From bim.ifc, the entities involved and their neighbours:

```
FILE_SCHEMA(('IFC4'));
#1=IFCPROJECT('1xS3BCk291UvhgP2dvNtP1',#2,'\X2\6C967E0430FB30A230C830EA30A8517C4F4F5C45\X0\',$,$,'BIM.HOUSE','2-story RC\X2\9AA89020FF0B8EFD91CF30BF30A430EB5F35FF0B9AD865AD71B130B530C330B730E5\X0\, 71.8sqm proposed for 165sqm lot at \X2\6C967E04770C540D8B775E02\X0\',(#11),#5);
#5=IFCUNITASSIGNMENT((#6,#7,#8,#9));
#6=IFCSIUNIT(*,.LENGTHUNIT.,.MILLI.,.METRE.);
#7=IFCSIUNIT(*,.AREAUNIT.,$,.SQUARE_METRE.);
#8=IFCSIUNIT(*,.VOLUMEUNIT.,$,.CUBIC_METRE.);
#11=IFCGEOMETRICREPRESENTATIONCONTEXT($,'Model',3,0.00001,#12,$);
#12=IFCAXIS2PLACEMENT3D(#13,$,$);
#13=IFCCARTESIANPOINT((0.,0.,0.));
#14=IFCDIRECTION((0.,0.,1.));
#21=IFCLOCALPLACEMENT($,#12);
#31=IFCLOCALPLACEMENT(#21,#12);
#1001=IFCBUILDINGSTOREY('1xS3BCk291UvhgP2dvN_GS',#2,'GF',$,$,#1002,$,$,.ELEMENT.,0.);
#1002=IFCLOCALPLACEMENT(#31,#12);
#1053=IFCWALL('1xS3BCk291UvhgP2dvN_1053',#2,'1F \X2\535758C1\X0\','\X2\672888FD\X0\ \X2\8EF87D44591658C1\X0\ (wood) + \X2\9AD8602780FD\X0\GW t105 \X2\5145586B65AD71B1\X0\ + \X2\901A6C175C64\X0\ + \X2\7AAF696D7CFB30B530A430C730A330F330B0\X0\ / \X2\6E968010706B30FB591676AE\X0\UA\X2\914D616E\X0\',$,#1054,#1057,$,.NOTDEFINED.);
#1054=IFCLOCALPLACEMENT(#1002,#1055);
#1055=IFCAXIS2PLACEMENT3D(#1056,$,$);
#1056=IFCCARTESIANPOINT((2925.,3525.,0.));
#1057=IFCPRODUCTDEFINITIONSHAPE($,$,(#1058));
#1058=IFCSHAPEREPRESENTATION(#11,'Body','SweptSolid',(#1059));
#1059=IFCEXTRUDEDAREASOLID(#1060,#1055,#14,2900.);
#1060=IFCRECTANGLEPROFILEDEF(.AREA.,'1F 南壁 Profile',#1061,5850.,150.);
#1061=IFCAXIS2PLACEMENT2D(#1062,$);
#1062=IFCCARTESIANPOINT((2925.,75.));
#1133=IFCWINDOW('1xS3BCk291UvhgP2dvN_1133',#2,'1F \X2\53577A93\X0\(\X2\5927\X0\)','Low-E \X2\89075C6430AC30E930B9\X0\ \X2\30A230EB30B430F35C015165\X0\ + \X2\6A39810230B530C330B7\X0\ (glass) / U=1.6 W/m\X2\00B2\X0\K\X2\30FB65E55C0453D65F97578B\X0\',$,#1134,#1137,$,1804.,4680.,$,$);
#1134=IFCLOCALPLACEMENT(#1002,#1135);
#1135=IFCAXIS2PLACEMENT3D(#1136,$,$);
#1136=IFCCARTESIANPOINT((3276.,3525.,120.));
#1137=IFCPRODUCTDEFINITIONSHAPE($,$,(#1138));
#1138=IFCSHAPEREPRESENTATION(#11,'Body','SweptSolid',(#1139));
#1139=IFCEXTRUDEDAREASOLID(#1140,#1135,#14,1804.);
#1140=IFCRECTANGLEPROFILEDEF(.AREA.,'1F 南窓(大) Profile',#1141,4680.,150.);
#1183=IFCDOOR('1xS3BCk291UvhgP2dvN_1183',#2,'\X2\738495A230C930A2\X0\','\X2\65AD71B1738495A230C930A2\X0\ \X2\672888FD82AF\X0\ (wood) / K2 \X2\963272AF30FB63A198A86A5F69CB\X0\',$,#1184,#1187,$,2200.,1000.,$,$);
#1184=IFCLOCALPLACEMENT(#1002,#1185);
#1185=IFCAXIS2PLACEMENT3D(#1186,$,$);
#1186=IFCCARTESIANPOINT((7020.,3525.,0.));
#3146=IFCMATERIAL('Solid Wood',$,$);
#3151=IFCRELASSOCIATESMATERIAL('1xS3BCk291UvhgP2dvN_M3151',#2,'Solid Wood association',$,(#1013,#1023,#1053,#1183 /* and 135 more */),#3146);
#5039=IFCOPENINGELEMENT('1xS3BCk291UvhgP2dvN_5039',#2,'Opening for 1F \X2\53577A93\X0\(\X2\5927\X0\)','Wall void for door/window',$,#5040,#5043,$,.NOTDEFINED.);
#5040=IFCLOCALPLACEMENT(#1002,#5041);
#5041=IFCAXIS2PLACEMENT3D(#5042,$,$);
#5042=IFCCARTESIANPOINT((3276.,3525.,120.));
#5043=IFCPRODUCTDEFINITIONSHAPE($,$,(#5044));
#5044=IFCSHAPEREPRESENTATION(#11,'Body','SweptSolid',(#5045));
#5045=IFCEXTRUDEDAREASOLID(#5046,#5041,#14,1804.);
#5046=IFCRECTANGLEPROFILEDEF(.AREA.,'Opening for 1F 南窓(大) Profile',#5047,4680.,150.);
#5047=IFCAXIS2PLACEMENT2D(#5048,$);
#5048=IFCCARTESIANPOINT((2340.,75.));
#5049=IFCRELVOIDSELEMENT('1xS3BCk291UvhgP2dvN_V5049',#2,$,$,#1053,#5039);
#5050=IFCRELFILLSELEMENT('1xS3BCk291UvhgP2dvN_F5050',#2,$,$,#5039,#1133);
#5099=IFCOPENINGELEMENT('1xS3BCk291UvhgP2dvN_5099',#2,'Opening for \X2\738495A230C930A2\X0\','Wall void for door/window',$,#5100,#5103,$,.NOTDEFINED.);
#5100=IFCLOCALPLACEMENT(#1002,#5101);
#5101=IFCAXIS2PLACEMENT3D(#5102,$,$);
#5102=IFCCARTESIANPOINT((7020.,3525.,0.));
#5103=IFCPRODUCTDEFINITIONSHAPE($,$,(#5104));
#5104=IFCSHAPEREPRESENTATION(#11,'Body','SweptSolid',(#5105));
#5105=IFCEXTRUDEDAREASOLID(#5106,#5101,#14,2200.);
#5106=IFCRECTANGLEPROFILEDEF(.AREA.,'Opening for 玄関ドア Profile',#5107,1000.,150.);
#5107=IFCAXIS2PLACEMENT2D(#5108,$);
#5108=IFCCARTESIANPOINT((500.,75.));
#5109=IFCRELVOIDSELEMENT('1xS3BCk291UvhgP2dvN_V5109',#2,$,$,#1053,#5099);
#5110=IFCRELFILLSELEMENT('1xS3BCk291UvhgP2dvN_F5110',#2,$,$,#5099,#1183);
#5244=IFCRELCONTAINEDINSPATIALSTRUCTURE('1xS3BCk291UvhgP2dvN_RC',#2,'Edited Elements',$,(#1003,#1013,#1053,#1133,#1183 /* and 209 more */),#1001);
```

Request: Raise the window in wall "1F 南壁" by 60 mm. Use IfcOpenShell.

```python
import numpy as np
import ifcopenshell
import ifcopenshell.api.geometry
import ifcopenshell.util.placement
import ifcopenshell.util.unit

model = ifcopenshell.open("bim.ifc")
unit_scale = ifcopenshell.util.unit.calculate_unit_scale(model)

window = model.by_guid("1xS3BCk291UvhgP2dvN_1133")
opening = window.FillsVoids[0].RelatingOpeningElement
dz = 0.06 / unit_scale

shift = np.array([0.0, 0.0, dz])
# The window is not placed relative to its opening, so move both.
for product in (opening, window):
    matrix = ifcopenshell.util.placement.get_local_placement(product.ObjectPlacement)
    matrix[:3, 3] += shift
    ifcopenshell.api.geometry.edit_object_placement(model, product=product, matrix=matrix, is_si=False)

print(f"moved by {dz * unit_scale:+.3f} m")

model.write("bim_edited.ifc")
```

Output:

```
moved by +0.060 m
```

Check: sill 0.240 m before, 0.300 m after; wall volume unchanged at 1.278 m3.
